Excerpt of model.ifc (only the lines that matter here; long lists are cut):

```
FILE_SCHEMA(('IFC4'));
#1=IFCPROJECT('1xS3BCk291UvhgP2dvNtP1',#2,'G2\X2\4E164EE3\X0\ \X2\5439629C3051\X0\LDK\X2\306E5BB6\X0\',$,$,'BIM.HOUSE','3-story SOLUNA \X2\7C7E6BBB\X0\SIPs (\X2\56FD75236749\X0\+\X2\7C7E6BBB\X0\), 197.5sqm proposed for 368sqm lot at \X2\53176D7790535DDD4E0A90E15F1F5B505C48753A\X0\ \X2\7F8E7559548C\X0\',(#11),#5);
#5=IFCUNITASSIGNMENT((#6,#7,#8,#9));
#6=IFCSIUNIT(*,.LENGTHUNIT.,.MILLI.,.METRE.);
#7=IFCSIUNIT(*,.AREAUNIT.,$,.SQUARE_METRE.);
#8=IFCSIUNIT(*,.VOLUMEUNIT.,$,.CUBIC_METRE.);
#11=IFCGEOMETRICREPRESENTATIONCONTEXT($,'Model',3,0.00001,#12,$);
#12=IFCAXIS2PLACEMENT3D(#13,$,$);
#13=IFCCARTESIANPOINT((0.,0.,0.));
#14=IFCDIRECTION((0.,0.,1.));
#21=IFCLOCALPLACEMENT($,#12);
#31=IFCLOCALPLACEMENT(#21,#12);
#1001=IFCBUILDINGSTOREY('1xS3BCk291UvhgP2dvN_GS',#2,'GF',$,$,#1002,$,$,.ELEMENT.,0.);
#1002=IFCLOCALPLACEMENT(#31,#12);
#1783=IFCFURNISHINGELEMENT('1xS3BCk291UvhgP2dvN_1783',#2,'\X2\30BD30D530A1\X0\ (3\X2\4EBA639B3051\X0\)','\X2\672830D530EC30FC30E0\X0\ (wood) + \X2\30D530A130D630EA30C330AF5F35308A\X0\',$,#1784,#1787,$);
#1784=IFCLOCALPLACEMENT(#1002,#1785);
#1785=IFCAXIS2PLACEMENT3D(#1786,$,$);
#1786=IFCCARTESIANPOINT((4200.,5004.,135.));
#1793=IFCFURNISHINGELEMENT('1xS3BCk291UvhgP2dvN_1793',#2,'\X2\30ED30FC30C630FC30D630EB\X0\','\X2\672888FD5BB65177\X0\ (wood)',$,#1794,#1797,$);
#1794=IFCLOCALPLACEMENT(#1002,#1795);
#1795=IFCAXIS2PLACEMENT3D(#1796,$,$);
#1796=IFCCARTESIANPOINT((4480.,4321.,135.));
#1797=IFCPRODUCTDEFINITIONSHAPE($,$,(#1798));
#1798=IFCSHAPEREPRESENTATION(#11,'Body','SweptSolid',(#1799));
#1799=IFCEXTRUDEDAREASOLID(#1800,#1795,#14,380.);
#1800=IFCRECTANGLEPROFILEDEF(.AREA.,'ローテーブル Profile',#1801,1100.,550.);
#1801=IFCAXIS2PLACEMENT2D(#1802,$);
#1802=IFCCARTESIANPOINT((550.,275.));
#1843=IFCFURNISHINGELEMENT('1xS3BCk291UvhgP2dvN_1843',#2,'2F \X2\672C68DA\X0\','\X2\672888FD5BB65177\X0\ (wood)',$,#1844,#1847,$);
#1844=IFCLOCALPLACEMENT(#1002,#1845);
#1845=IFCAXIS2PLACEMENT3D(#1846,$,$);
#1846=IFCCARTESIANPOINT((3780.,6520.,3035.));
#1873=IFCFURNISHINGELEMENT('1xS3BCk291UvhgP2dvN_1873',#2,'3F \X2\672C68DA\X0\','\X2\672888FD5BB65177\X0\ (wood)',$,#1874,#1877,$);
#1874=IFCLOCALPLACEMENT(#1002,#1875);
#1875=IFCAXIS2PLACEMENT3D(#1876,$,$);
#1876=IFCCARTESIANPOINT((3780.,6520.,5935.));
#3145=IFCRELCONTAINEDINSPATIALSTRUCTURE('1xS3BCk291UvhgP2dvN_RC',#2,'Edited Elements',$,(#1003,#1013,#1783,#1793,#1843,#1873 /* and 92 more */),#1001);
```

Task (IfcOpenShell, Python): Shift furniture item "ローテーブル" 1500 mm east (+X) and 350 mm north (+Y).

```python
import ifcopenshell
import ifcopenshell.api.geometry
import ifcopenshell.util.placement

model = ifcopenshell.open("model.ifc")

item = model.by_guid("1xS3BCk291UvhgP2dvN_1793")
matrix = ifcopenshell.util.placement.get_local_placement(item.ObjectPlacement)
matrix[0, 3] += 1500.0
matrix[1, 3] += 350.0
ifcopenshell.api.geometry.edit_object_placement(model, product=item, matrix=matrix, is_si=False)

print(ifcopenshell.util.placement.get_local_placement(item.ObjectPlacement).round(3) + 0.0)

model.write("model_updated.ifc")
```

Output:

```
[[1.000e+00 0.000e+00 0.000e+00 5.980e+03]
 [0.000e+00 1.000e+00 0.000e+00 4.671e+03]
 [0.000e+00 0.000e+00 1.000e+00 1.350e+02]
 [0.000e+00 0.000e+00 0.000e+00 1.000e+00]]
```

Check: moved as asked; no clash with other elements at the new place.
